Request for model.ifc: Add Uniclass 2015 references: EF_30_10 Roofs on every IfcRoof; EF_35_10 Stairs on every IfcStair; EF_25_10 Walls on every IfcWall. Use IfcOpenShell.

First a look at what the model holds.

```python
import ifcopenshell

model = ifcopenshell.open("model.ifc")
print(model.schema)
print("classifications:", [c.Name for c in model.by_type("IfcClassification")])
for ifc_class in ("IfcDoor", "IfcRoof", "IfcStair", "IfcWall", "IfcWindow"):
    print(ifc_class, len(model.by_type(ifc_class)))
```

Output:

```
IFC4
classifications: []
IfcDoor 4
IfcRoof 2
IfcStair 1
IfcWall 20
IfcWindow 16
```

```python
import ifcopenshell
import ifcopenshell.api.classification

model = ifcopenshell.open("model.ifc")

system = ifcopenshell.api.classification.add_classification(model, classification="Uniclass 2015")

codes = {
    "IfcRoof": ("EF_30_10", "Roofs"),
    "IfcStair": ("EF_35_10", "Stairs"),
    "IfcWall": ("EF_25_10", "Walls"),
}
for ifc_class, (code, name) in codes.items():
    products = model.by_type(ifc_class)
    ifcopenshell.api.classification.add_reference(
        model, products=products, classification=system, identification=code, name=name
    )
    print(code, len(products))

model.write("model_v2.ifc")
```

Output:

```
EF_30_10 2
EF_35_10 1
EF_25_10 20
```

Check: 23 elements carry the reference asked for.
